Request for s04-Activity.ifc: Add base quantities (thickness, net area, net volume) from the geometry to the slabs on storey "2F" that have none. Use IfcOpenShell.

First a look at what the model holds.

```python
import ifcopenshell
import ifcopenshell.util.element
import ifcopenshell.util.unit

model = ifcopenshell.open("s04-Activity.ifc")
print(model.schema)
for unit_type in ("LENGTHUNIT", "AREAUNIT", "VOLUMEUNIT"):
    print(unit_type, ifcopenshell.util.unit.calculate_unit_scale(model, unit_type))
storey = next(s for s in model.by_type("IfcBuildingStorey") if s.Name == "2F")
slabs = [e for e in ifcopenshell.util.element.get_decomposition(storey) if e.is_a("IfcSlab")]
for e in sorted(slabs, key=lambda e: e.id()):
    print(e.id(), e.is_a(), e.Name, list(ifcopenshell.util.element.get_psets(e, qtos_only=True)), sep=" | ")
```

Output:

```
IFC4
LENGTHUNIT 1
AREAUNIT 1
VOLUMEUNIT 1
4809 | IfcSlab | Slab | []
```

```python
import ifcopenshell
import ifcopenshell.api.pset
import ifcopenshell.geom
import ifcopenshell.util.element
import ifcopenshell.util.shape
import ifcopenshell.util.unit

model = ifcopenshell.open("s04-Activity.ifc")
unit_scale = ifcopenshell.util.unit.calculate_unit_scale(model)
area_scale = ifcopenshell.util.unit.calculate_unit_scale(model, "AREAUNIT")
volume_scale = ifcopenshell.util.unit.calculate_unit_scale(model, "VOLUMEUNIT")
settings = ifcopenshell.geom.settings()

storey = next(s for s in model.by_type("IfcBuildingStorey") if s.Name == "2F")
slabs = [e for e in ifcopenshell.util.element.get_decomposition(storey) if e.is_a("IfcSlab")]

for e in sorted(slabs, key=lambda e: e.id()):
    if ifcopenshell.util.element.get_psets(e, qtos_only=True, should_inherit=False):
        continue
    # Geometry comes back in metres, in the element's own axes.
    shape = ifcopenshell.geom.create_shape(settings, e)
    values = {
        "Width": ifcopenshell.util.shape.get_z(shape.geometry) / unit_scale,
        "NetArea": ifcopenshell.util.shape.get_footprint_area(shape.geometry) / area_scale,
        "NetVolume": ifcopenshell.util.shape.get_volume(shape.geometry) / volume_scale,
    }
    qto = ifcopenshell.api.pset.add_qto(model, product=e, name="Qto_SlabBaseQuantities")
    ifcopenshell.api.pset.edit_qto(model, qto=qto, properties=values)
    print(e.id(), {k: round(v, 3) for k, v in values.items()})

model.write("s04-Activity_updated.ifc")
```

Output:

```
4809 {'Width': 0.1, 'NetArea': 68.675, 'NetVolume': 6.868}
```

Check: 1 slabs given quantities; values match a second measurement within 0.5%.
